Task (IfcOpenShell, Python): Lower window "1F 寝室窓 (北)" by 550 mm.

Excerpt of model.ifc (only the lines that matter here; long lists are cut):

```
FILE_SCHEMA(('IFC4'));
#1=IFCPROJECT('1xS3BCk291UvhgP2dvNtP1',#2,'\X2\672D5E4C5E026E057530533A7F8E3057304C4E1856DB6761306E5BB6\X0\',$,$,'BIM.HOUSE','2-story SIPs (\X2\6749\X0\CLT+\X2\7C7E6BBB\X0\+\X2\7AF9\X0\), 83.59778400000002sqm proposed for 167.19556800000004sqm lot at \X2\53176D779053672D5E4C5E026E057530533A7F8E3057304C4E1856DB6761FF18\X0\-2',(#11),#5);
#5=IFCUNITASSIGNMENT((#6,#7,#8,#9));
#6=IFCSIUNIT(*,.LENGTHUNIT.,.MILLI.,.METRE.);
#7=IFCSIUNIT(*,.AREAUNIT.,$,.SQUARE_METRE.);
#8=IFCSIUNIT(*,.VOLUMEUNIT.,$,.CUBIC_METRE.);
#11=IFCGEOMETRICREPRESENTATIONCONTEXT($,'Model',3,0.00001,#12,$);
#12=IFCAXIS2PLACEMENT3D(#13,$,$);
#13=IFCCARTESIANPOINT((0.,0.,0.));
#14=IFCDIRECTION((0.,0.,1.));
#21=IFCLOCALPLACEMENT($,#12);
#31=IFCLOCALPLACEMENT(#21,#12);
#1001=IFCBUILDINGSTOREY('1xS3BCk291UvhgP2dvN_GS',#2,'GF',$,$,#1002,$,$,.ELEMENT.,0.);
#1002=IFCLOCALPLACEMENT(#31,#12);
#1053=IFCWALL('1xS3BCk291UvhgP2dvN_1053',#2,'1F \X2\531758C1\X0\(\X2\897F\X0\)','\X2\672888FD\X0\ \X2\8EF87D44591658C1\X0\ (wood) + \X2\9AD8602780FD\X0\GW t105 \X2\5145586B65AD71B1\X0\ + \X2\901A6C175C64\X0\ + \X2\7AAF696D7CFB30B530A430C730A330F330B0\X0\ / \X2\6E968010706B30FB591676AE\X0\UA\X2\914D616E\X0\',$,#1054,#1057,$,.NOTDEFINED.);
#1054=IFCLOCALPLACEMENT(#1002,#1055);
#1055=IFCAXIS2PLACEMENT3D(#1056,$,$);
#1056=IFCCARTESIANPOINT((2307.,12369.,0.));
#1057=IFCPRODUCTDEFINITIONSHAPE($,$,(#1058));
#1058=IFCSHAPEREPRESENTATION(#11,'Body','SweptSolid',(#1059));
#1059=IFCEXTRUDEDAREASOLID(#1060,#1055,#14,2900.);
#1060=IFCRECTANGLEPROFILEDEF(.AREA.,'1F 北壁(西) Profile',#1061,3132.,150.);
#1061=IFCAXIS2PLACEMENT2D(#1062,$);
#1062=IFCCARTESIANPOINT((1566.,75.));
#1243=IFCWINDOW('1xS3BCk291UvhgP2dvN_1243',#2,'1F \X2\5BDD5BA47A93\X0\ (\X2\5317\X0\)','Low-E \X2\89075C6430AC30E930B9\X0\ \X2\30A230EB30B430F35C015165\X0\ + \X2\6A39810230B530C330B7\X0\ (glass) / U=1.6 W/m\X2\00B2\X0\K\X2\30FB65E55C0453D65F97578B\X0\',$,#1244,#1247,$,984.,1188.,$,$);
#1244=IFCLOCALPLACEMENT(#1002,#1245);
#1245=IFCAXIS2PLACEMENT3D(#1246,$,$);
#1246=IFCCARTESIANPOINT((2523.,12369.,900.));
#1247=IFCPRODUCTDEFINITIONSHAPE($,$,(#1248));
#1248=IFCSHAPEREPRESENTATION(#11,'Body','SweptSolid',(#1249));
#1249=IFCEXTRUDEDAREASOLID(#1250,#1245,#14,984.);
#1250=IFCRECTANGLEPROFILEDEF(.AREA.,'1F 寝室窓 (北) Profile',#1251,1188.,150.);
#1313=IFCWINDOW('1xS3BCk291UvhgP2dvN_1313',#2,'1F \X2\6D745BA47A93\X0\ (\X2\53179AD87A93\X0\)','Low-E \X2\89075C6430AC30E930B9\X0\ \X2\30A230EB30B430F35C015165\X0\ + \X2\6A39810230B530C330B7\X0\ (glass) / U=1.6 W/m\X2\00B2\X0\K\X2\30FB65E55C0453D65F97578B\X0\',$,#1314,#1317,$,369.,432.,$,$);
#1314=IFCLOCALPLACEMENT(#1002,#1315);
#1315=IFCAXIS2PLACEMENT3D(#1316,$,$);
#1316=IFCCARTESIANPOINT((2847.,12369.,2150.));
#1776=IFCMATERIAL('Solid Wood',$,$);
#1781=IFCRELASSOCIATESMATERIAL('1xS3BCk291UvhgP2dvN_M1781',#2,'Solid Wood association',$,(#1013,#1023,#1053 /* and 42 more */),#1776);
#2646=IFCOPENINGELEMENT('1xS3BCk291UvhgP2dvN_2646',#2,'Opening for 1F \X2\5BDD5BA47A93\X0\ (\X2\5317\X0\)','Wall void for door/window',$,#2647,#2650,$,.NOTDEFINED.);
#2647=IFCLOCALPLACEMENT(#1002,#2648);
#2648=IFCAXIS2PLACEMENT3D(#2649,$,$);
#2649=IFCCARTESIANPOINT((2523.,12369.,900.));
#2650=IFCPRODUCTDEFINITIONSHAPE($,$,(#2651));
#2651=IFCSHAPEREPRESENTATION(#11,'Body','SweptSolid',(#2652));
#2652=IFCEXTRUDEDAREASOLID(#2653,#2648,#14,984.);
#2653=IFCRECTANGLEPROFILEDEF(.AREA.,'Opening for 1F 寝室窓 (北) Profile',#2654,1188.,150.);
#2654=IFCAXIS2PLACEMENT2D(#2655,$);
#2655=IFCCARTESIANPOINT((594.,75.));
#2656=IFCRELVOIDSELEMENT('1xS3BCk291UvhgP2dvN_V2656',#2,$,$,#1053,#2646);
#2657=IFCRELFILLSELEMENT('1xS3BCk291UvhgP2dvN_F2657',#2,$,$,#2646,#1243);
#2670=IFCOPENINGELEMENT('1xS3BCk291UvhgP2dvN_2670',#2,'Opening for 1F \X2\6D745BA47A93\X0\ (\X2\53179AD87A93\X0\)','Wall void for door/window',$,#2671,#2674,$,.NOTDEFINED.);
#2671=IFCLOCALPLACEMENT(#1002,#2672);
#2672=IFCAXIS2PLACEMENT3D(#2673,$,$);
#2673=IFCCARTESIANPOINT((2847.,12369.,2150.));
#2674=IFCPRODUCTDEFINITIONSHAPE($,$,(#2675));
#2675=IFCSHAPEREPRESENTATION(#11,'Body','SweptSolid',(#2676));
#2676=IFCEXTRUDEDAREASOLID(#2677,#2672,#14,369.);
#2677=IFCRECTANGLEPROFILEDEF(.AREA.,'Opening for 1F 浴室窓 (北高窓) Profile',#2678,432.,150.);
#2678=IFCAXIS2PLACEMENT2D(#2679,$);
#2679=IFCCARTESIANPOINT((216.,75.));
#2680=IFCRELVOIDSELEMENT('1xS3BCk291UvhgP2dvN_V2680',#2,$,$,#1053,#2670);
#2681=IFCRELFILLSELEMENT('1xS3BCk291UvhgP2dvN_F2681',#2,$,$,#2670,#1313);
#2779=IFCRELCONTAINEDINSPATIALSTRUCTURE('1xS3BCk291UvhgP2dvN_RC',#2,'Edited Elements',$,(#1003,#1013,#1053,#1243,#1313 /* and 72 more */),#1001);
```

```python
import numpy as np
import ifcopenshell
import ifcopenshell.api.geometry
import ifcopenshell.util.placement
import ifcopenshell.util.unit

model = ifcopenshell.open("model.ifc")
unit_scale = ifcopenshell.util.unit.calculate_unit_scale(model)

window = model.by_guid("1xS3BCk291UvhgP2dvN_1243")
opening = window.FillsVoids[0].RelatingOpeningElement
dz = -0.55 / unit_scale

shift = np.array([0.0, 0.0, dz])
# The window is not placed relative to its opening, so move both.
for product in (opening, window):
    matrix = ifcopenshell.util.placement.get_local_placement(product.ObjectPlacement)
    matrix[:3, 3] += shift
    ifcopenshell.api.geometry.edit_object_placement(model, product=product, matrix=matrix, is_si=False)

print(f"moved by {dz * unit_scale:+.3f} m")

model.write("model_updated.ifc")
```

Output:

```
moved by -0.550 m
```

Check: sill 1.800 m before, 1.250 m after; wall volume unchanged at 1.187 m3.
